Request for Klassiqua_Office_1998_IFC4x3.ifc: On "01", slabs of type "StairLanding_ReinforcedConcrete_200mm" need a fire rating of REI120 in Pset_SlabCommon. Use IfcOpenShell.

First a look at what the model holds.

```python
import ifcopenshell
import ifcopenshell.util.element

model = ifcopenshell.open("Klassiqua_Office_1998_IFC4x3.ifc")
print(model.schema)
storey = next(s for s in model.by_type("IfcBuildingStorey") if s.Name == "01")
slabs = [e for e in ifcopenshell.util.element.get_decomposition(storey) if e.is_a("IfcSlab")]
seen = {}
for e in slabs:
    element_type = ifcopenshell.util.element.get_type(e)
    key = (element_type.Name if element_type != e and element_type else None, ifcopenshell.util.element.get_pset(e, "Pset_SlabCommon", "FireRating"))
    seen[key] = seen.get(key, 0) + 1
for (name, value), count in sorted(seen.items(), key=str):
    print(count, "x", name, "|", value)
```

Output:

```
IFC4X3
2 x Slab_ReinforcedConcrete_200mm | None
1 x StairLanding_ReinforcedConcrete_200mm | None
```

```python
import ifcopenshell
import ifcopenshell.api.pset
import ifcopenshell.util.element

model = ifcopenshell.open("Klassiqua_Office_1998_IFC4x3.ifc")

storey = next(s for s in model.by_type("IfcBuildingStorey") if s.Name == "01")
slabs = [e for e in ifcopenshell.util.element.get_decomposition(storey) if e.is_a("IfcSlab")]

count = 0
for e in slabs:
    element_type = ifcopenshell.util.element.get_type(e)
    if element_type in (None, e) or element_type.Name != "StairLanding_ReinforcedConcrete_200mm":
        continue
    # add_pset returns the element's existing set when there is one.
    pset = ifcopenshell.api.pset.add_pset(model, product=e, name="Pset_SlabCommon")
    ifcopenshell.api.pset.edit_pset(model, pset=pset, properties={"FireRating": "REI120"})
    count += 1

print(count, "slabs updated")

model.write("Klassiqua_Office_1998_IFC4x3_updated.ifc")
```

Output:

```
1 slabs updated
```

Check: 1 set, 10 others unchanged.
